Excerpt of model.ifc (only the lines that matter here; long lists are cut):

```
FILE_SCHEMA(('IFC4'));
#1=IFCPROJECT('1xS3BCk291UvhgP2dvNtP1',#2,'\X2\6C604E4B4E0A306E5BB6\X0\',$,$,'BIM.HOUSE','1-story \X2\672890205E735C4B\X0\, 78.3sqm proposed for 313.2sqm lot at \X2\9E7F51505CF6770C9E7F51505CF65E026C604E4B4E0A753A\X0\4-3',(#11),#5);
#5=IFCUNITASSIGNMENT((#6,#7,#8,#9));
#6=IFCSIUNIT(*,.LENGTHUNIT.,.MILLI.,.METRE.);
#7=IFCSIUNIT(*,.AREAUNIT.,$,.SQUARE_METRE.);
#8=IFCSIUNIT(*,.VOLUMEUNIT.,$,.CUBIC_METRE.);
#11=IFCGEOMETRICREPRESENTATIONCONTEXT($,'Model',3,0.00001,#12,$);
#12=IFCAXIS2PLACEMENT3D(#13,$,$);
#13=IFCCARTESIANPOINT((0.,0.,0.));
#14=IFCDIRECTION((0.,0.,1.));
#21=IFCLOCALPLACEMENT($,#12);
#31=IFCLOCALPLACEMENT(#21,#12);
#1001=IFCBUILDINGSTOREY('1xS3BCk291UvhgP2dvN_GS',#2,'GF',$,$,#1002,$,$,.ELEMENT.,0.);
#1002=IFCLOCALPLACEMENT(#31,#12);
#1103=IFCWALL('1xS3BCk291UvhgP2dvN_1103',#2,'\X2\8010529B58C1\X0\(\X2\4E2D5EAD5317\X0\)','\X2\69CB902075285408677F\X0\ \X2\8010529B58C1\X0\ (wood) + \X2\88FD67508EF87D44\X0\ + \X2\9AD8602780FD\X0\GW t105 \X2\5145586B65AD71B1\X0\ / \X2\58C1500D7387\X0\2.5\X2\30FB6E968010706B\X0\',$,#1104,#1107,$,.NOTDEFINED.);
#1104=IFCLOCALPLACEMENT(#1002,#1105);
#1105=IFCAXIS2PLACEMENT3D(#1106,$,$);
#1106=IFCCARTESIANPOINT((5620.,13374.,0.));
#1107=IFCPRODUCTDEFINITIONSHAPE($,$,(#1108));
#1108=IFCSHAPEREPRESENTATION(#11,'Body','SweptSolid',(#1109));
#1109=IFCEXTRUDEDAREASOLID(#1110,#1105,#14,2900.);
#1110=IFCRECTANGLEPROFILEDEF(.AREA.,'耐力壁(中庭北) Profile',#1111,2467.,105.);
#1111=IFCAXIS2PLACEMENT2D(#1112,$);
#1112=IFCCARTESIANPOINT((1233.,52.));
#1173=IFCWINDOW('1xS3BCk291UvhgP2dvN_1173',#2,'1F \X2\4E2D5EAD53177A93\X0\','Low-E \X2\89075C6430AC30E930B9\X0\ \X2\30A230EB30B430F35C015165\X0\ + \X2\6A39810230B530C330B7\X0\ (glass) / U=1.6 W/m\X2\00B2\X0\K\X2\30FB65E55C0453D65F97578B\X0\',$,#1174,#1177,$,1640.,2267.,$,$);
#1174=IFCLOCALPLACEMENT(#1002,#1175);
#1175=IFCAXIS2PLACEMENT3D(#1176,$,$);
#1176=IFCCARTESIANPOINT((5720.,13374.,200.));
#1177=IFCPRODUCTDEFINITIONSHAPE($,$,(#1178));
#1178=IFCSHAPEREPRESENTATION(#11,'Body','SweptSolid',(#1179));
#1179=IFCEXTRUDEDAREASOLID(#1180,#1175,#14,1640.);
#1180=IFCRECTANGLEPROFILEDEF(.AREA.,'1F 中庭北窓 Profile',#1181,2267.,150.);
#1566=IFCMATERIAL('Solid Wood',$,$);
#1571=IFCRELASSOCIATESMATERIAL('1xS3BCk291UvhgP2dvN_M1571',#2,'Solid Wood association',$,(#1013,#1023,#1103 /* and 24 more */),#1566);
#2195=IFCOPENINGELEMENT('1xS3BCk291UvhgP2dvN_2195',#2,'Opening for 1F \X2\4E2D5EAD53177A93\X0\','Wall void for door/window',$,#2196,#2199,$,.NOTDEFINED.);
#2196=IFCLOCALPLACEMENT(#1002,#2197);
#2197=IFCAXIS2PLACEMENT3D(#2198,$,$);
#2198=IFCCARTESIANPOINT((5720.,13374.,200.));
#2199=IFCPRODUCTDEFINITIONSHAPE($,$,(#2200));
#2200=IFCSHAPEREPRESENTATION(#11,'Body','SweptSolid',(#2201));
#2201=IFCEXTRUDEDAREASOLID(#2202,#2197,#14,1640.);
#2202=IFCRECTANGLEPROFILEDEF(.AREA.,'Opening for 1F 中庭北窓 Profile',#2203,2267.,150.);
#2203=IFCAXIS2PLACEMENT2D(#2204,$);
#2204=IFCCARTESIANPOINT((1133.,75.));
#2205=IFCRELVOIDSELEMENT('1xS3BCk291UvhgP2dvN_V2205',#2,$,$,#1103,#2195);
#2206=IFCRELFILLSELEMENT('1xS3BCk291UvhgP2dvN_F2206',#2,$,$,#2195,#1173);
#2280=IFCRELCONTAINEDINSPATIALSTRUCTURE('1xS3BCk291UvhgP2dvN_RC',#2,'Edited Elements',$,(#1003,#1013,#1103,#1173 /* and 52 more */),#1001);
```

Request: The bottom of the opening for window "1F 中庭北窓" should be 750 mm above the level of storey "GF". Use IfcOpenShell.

```python
import numpy as np
import ifcopenshell
import ifcopenshell.api.geometry
import ifcopenshell.geom
import ifcopenshell.util.element
import ifcopenshell.util.placement
import ifcopenshell.util.shape
import ifcopenshell.util.unit

model = ifcopenshell.open("model.ifc")
unit_scale = ifcopenshell.util.unit.calculate_unit_scale(model)

window = model.by_id(1173)
opening = window.FillsVoids[0].RelatingOpeningElement
storey = ifcopenshell.util.element.get_container(window, ifc_class="IfcBuildingStorey")
level = ifcopenshell.util.placement.get_local_placement(storey.ObjectPlacement)[2, 3]

# The opening's origin need not be at the sill, so measure its lowest point.
shape = ifcopenshell.geom.create_shape(ifcopenshell.geom.settings(), opening)
bottom = ifcopenshell.util.shape.get_shape_bottom_elevation(shape, shape.geometry) / unit_scale
dz = level + 0.75 / unit_scale - bottom

shift = np.array([0.0, 0.0, dz])
# The window is not placed relative to its opening, so move both.
for product in (opening, window):
    matrix = ifcopenshell.util.placement.get_local_placement(product.ObjectPlacement)
    matrix[:3, 3] += shift
    ifcopenshell.api.geometry.edit_object_placement(model, product=product, matrix=matrix, is_si=False)

print(f"moved by {dz * unit_scale:+.3f} m")

model.write("model_rev.ifc")
```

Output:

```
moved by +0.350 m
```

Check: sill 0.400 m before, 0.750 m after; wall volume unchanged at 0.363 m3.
